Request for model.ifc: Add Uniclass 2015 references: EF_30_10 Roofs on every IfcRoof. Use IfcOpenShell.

First a look at what the model holds.

```python
import ifcopenshell

model = ifcopenshell.open("model.ifc")
print(model.schema)
print("classifications:", [c.Name for c in model.by_type("IfcClassification")])
for ifc_class in ("IfcDoor", "IfcRoof", "IfcStair", "IfcWall", "IfcWindow"):
    print(ifc_class, len(model.by_type(ifc_class)))
```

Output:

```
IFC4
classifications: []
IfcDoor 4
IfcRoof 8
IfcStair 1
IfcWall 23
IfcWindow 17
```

```python
import ifcopenshell
import ifcopenshell.api.classification

model = ifcopenshell.open("model.ifc")

system = ifcopenshell.api.classification.add_classification(model, classification="Uniclass 2015")

codes = {
    "IfcRoof": ("EF_30_10", "Roofs"),
}
for ifc_class, (code, name) in codes.items():
    products = model.by_type(ifc_class)
    ifcopenshell.api.classification.add_reference(
        model, products=products, classification=system, identification=code, name=name
    )
    print(code, len(products))

model.write("model_updated.ifc")
```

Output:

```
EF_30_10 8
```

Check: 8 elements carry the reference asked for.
